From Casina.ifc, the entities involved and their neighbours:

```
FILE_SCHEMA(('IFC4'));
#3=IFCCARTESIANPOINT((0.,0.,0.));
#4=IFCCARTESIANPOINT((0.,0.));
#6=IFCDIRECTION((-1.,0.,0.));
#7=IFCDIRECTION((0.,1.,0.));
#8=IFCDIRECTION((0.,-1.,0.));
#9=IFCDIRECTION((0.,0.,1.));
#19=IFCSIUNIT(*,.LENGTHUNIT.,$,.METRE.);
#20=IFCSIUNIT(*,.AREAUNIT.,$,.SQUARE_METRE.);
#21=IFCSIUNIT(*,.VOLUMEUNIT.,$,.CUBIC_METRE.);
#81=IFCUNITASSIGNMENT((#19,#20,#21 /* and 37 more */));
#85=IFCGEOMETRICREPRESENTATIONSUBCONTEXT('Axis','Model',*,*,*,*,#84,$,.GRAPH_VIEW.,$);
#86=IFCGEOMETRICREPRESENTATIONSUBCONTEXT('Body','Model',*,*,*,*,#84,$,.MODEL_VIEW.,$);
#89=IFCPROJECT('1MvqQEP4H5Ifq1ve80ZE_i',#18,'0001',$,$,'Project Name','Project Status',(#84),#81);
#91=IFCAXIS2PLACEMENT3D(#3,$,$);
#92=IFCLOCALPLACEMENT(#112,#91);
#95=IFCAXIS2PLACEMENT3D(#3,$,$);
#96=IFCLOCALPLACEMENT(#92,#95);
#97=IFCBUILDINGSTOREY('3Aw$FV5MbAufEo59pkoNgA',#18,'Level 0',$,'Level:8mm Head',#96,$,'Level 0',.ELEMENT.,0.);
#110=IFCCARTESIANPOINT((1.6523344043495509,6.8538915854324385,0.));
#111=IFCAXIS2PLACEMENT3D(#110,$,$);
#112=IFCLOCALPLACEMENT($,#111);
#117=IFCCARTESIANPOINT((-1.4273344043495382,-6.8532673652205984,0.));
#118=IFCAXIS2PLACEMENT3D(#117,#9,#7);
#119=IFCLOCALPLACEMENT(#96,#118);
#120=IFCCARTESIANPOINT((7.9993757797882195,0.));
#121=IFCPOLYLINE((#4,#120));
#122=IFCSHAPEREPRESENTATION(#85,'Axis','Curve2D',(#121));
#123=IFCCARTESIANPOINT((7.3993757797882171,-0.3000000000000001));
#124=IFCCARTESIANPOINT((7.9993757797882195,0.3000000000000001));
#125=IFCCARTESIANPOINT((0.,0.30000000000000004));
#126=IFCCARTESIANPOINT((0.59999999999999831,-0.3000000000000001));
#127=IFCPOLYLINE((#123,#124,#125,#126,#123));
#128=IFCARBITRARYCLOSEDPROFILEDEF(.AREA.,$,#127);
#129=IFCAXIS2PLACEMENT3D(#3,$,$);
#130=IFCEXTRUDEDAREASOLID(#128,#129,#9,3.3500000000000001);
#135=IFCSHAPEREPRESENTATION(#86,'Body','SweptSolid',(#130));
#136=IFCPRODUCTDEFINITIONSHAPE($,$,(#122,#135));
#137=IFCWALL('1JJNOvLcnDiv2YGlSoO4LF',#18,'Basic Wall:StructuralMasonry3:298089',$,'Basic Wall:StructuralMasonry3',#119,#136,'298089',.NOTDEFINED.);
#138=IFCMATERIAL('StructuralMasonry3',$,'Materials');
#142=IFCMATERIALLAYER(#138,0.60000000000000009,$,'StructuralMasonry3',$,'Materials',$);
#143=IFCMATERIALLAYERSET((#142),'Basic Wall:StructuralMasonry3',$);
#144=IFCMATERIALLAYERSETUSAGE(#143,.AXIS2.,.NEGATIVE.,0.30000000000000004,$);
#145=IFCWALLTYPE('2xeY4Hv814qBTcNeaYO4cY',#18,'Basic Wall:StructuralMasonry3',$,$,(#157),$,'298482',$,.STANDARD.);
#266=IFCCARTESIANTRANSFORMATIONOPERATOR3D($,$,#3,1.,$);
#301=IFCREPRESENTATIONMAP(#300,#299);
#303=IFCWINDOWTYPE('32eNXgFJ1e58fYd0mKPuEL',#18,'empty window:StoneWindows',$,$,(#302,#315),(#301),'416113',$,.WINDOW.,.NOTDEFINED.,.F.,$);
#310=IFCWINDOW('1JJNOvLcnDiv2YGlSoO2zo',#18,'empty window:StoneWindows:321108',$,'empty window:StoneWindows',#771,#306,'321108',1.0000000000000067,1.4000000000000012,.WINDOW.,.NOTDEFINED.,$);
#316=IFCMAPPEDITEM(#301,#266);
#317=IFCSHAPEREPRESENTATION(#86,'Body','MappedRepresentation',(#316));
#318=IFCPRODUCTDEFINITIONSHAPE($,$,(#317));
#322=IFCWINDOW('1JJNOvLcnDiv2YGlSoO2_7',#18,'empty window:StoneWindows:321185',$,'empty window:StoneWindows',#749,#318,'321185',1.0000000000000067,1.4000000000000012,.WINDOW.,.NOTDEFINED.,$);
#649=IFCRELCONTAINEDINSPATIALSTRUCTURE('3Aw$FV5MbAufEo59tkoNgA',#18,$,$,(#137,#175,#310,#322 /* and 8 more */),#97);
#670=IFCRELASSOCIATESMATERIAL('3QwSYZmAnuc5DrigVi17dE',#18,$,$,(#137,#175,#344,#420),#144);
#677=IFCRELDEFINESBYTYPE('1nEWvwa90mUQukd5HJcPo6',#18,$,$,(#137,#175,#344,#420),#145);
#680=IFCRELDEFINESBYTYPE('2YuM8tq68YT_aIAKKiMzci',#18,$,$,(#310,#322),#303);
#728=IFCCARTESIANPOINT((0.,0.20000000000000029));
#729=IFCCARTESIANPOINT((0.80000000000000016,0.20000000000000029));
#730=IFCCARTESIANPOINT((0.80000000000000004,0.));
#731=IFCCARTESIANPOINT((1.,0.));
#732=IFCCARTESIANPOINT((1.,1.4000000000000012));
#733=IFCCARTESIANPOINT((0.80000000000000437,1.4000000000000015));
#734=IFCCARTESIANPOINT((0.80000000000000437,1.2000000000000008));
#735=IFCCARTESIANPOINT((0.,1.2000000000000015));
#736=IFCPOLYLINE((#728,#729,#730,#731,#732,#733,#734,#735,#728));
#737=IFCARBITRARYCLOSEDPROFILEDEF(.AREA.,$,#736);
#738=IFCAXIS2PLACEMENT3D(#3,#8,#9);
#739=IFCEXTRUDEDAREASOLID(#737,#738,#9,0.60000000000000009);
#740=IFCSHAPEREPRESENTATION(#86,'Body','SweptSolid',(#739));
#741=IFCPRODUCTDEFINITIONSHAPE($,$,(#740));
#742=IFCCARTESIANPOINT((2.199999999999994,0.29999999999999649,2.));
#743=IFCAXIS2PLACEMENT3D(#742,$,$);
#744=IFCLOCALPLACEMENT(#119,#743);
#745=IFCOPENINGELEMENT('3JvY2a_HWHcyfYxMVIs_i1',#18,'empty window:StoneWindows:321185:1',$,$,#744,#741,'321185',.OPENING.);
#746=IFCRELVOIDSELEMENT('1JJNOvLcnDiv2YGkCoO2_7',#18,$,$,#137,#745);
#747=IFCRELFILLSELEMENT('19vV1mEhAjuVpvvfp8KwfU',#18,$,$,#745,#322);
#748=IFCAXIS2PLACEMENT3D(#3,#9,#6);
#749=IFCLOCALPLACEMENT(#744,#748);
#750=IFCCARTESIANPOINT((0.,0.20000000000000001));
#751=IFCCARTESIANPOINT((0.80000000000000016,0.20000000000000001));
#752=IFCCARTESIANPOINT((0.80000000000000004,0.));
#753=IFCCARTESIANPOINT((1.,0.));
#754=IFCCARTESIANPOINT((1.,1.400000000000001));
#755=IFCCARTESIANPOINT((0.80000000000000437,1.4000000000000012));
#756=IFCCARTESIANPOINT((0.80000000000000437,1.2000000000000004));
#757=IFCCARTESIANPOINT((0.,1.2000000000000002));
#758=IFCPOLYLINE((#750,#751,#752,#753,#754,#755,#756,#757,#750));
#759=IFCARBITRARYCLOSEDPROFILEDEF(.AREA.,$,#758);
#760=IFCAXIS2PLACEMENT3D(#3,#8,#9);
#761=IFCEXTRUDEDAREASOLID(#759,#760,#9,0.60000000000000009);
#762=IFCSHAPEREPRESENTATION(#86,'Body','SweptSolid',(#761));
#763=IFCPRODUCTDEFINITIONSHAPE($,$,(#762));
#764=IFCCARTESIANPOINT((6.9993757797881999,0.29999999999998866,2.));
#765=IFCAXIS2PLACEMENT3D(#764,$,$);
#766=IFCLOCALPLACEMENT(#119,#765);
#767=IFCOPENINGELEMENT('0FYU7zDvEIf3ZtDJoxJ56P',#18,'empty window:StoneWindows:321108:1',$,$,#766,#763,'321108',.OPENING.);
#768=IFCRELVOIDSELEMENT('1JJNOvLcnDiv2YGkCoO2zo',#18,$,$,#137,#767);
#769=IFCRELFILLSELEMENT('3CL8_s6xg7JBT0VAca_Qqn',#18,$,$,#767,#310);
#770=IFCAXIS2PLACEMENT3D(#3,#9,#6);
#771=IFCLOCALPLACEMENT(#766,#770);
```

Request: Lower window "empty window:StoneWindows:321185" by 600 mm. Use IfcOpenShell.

```python
import numpy as np
import ifcopenshell
import ifcopenshell.api.geometry
import ifcopenshell.util.placement
import ifcopenshell.util.unit

model = ifcopenshell.open("Casina.ifc")
unit_scale = ifcopenshell.util.unit.calculate_unit_scale(model)

window = model.by_guid("1JJNOvLcnDiv2YGlSoO2_7")
opening = window.FillsVoids[0].RelatingOpeningElement
dz = -0.6 / unit_scale

shift = np.array([0.0, 0.0, dz])
# The window is placed relative to its opening, so it follows when the opening moves.
matrix = ifcopenshell.util.placement.get_local_placement(opening.ObjectPlacement)
matrix[:3, 3] += shift
ifcopenshell.api.geometry.edit_object_placement(
    model, product=opening, matrix=matrix, is_si=False, should_transform_children=True
)

print(f"moved by {dz * unit_scale:+.3f} m")

model.write("Casina_updated.ifc")
```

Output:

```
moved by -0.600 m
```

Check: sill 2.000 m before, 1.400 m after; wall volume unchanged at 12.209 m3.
